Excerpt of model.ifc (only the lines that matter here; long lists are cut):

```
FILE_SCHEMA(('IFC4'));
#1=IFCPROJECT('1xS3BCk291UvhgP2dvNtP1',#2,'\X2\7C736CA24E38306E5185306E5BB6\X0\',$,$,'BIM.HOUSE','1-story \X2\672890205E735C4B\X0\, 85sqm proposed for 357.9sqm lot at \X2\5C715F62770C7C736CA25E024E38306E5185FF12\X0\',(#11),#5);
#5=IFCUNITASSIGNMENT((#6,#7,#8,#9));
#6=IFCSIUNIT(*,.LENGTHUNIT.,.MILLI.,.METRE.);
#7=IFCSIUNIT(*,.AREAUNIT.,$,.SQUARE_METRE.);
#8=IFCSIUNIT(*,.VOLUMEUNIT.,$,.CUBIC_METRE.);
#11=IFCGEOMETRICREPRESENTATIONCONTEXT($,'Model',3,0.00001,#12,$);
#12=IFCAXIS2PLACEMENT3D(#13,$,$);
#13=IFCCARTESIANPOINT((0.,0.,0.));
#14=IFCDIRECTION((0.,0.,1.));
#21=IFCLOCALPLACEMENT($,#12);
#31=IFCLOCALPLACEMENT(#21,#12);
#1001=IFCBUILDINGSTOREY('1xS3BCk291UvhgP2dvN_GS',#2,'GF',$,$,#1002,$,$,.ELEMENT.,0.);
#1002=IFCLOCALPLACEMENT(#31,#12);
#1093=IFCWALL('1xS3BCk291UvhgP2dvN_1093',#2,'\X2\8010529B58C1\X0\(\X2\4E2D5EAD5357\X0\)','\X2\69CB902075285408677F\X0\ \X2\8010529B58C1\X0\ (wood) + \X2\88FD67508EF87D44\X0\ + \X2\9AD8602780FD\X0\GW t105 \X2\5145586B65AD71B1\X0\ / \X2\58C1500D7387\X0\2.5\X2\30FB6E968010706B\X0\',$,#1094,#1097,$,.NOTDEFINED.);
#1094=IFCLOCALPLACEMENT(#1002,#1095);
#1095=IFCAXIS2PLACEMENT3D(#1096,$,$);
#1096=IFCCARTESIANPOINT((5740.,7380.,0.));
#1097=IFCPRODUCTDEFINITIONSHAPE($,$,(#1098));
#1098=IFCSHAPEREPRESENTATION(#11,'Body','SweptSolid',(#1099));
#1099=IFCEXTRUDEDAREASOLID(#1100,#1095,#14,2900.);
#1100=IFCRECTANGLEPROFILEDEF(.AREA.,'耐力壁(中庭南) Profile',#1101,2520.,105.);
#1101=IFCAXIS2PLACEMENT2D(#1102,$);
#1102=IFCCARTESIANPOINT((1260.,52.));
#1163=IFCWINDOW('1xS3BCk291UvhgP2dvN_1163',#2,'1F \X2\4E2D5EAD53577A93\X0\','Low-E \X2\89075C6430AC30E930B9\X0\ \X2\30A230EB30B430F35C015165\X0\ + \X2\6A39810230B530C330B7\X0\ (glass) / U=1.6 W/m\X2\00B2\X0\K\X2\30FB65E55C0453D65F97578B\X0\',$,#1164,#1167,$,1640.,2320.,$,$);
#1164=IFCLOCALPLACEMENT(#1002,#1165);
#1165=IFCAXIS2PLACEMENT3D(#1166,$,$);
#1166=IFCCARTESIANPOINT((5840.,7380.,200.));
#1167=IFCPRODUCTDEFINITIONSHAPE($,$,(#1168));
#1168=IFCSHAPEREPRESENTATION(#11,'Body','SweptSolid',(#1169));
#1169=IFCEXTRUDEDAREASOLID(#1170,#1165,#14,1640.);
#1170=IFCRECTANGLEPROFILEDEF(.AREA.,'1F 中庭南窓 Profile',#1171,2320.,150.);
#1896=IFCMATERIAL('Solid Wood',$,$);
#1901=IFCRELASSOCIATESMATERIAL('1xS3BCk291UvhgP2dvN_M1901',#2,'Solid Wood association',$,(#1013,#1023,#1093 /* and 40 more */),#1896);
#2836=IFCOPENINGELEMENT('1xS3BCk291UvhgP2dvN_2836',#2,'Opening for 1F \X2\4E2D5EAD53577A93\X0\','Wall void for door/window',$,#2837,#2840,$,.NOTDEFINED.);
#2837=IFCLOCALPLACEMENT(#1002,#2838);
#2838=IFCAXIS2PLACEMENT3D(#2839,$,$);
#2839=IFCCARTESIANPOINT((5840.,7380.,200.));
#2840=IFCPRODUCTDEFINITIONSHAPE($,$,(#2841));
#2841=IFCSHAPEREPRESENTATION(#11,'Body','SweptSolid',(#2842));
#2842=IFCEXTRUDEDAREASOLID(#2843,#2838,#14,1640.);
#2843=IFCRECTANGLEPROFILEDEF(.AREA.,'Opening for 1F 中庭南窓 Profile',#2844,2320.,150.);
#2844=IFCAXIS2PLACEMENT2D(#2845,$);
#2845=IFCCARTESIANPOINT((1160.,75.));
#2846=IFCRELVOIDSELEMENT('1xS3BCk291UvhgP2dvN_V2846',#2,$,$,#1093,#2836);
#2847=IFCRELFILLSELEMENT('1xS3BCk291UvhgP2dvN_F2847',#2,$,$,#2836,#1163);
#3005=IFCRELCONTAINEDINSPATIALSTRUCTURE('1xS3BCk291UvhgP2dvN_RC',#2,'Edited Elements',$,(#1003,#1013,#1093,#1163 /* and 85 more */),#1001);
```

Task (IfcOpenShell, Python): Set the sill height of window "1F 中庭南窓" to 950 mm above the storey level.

```python
import numpy as np
import ifcopenshell
import ifcopenshell.api.geometry
import ifcopenshell.geom
import ifcopenshell.util.element
import ifcopenshell.util.placement
import ifcopenshell.util.shape
import ifcopenshell.util.unit

model = ifcopenshell.open("model.ifc")
unit_scale = ifcopenshell.util.unit.calculate_unit_scale(model)

window = model.by_guid("1xS3BCk291UvhgP2dvN_1163")
opening = window.FillsVoids[0].RelatingOpeningElement
storey = ifcopenshell.util.element.get_container(window, ifc_class="IfcBuildingStorey")
level = ifcopenshell.util.placement.get_local_placement(storey.ObjectPlacement)[2, 3]

# The opening's origin need not be at the sill, so measure its lowest point.
shape = ifcopenshell.geom.create_shape(ifcopenshell.geom.settings(), opening)
bottom = ifcopenshell.util.shape.get_shape_bottom_elevation(shape, shape.geometry) / unit_scale
dz = level + 0.95 / unit_scale - bottom

shift = np.array([0.0, 0.0, dz])
# The window is not placed relative to its opening, so move both.
for product in (opening, window):
    matrix = ifcopenshell.util.placement.get_local_placement(product.ObjectPlacement)
    matrix[:3, 3] += shift
    ifcopenshell.api.geometry.edit_object_placement(model, product=product, matrix=matrix, is_si=False)

print(f"moved by {dz * unit_scale:+.3f} m")

model.write("model_v2.ifc")
```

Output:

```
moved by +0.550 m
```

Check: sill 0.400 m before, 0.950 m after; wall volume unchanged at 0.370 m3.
